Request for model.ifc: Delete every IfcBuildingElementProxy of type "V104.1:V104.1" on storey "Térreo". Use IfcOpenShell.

First a look at what the model holds.

```python
import ifcopenshell
import ifcopenshell.util.element

model = ifcopenshell.open("model.ifc")
print(model.schema)
storey = next(s for s in model.by_type("IfcBuildingStorey") if s.Name == "Térreo")
proxies = [e for e in ifcopenshell.util.element.get_decomposition(storey) if e.is_a("IfcBuildingElementProxy")]
seen = {}
for e in proxies:
    element_type = ifcopenshell.util.element.get_type(e)
    name = element_type.Name if element_type not in (None, e) else None
    seen[name] = seen.get(name, 0) + 1
for name, count in sorted(seen.items(), key=str):
    print(count, "x", name)
```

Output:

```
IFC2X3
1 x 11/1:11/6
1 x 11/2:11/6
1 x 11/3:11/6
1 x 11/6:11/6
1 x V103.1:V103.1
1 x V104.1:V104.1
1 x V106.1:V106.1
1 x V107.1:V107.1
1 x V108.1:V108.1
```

```python
import ifcopenshell
import ifcopenshell.api.root
import ifcopenshell.util.element

model = ifcopenshell.open("model.ifc")

storey = next(s for s in model.by_type("IfcBuildingStorey") if s.Name == "Térreo")
proxies = [e for e in ifcopenshell.util.element.get_decomposition(storey) if e.is_a("IfcBuildingElementProxy")]
targets = [e for e in proxies if (t := ifcopenshell.util.element.get_type(e)) not in (None, e) and t.Name == "V104.1:V104.1"]

for e in targets:
    ifcopenshell.api.root.remove_product(model, product=e)
print(len(targets), "removed")

model.write("model_updated.ifc")
```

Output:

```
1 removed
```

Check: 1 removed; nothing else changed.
